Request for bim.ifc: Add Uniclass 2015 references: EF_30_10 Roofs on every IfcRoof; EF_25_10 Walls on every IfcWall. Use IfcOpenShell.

First a look at what the model holds.

```python
import ifcopenshell

model = ifcopenshell.open("bim.ifc")
print(model.schema)
print("classifications:", [c.Name for c in model.by_type("IfcClassification")])
for ifc_class in ("IfcDoor", "IfcRoof", "IfcStair", "IfcWall", "IfcWindow"):
    print(ifc_class, len(model.by_type(ifc_class)))
```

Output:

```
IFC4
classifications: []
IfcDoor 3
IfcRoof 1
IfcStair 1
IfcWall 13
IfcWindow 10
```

```python
import ifcopenshell
import ifcopenshell.api.classification

model = ifcopenshell.open("bim.ifc")

system = ifcopenshell.api.classification.add_classification(model, classification="Uniclass 2015")

codes = {
    "IfcRoof": ("EF_30_10", "Roofs"),
    "IfcWall": ("EF_25_10", "Walls"),
}
for ifc_class, (code, name) in codes.items():
    products = model.by_type(ifc_class)
    ifcopenshell.api.classification.add_reference(
        model, products=products, classification=system, identification=code, name=name
    )
    print(code, len(products))

model.write("bim_v2.ifc")
```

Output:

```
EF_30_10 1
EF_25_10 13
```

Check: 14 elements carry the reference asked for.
